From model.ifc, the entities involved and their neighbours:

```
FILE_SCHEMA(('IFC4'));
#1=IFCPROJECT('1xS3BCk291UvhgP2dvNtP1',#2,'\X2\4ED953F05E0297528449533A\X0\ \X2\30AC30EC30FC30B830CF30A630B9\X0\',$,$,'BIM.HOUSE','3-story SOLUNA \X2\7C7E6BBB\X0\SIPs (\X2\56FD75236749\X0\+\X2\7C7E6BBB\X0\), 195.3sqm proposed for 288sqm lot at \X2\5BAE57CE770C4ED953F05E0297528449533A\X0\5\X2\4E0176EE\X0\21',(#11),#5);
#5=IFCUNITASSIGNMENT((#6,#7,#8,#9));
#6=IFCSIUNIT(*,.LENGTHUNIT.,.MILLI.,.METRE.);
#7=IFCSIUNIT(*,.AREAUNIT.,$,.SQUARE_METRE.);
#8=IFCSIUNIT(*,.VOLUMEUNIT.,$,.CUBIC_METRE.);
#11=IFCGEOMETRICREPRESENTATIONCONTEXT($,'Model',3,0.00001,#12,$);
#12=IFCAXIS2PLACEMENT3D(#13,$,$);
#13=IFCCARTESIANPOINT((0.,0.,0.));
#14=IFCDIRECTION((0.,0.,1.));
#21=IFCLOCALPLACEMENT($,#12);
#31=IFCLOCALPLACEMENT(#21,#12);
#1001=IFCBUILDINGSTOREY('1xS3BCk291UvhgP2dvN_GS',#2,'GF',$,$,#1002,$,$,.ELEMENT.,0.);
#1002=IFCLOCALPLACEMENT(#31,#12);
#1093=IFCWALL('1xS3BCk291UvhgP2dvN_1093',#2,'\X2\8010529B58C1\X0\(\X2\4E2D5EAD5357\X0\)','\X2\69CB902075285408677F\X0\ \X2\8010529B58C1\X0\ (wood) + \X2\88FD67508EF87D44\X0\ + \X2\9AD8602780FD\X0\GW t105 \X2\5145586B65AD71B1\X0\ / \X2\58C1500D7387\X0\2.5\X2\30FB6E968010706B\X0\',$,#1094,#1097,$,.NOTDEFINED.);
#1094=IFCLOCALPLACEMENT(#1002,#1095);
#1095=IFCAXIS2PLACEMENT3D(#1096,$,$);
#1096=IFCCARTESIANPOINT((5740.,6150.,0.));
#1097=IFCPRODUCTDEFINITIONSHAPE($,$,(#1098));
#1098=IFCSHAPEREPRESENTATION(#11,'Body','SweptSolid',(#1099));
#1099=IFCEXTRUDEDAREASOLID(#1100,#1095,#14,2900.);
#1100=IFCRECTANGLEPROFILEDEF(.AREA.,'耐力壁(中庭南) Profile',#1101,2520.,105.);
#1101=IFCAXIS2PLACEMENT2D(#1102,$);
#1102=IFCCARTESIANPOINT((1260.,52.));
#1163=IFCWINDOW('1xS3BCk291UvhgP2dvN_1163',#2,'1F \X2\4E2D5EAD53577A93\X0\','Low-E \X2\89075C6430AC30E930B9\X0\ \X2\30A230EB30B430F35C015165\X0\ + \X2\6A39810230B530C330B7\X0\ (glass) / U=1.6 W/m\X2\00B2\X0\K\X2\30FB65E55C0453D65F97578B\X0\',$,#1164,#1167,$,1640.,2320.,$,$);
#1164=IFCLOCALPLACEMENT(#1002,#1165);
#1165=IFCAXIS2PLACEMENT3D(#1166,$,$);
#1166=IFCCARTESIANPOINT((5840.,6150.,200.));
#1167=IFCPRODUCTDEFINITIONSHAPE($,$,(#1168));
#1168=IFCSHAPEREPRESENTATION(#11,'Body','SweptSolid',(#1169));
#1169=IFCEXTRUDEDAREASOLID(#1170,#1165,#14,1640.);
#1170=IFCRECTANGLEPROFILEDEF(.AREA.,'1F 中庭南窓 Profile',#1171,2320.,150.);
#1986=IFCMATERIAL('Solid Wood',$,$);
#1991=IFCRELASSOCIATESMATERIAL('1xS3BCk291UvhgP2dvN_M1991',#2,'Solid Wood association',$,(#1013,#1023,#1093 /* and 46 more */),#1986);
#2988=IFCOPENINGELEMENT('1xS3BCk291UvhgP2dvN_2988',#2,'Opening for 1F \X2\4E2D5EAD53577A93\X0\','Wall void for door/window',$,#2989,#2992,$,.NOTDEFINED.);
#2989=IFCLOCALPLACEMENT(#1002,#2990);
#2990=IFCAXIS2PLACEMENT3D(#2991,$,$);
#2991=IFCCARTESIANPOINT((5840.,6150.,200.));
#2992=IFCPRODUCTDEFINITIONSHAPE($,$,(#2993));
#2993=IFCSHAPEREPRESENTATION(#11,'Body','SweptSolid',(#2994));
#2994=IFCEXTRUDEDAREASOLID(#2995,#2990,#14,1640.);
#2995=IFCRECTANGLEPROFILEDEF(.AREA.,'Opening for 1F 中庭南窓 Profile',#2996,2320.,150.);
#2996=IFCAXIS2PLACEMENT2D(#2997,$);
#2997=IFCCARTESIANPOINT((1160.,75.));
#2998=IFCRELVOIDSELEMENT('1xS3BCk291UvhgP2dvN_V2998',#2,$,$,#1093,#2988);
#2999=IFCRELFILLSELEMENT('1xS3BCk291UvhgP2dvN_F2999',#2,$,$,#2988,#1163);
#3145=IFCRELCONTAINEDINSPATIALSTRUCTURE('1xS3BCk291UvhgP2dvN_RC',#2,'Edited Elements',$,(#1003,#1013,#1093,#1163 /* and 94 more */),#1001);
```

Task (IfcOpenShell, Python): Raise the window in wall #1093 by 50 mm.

```python
import numpy as np
import ifcopenshell
import ifcopenshell.api.geometry
import ifcopenshell.util.placement
import ifcopenshell.util.unit

model = ifcopenshell.open("model.ifc")
unit_scale = ifcopenshell.util.unit.calculate_unit_scale(model)

window = model.by_guid("1xS3BCk291UvhgP2dvN_1163")
opening = window.FillsVoids[0].RelatingOpeningElement
dz = 0.05 / unit_scale

shift = np.array([0.0, 0.0, dz])
# The window is not placed relative to its opening, so move both.
for product in (opening, window):
    matrix = ifcopenshell.util.placement.get_local_placement(product.ObjectPlacement)
    matrix[:3, 3] += shift
    ifcopenshell.api.geometry.edit_object_placement(model, product=product, matrix=matrix, is_si=False)

print(f"moved by {dz * unit_scale:+.3f} m")

model.write("model_v2.ifc")
```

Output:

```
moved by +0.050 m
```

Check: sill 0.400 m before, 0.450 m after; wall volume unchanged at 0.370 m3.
